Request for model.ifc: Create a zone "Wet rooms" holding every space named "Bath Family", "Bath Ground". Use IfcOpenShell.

First a look at what the model holds.

```python
import ifcopenshell

model = ifcopenshell.open("model.ifc")
print(model.schema)
seen = {}
for space in model.by_type("IfcSpace"):
    seen[space.LongName] = seen.get(space.LongName, 0) + 1
for name, count in sorted(seen.items(), key=str):
    print(count, "x", name)
print("zones:", [z.Name for z in model.by_type("IfcZone")][:20])
```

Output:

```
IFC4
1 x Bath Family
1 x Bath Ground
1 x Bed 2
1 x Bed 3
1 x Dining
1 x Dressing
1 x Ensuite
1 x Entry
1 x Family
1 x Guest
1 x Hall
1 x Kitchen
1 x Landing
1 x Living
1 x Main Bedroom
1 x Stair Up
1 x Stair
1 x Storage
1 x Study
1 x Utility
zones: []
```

```python
import ifcopenshell
import ifcopenshell.api.group
import ifcopenshell.api.root

model = ifcopenshell.open("model.ifc")

names = {"Bath Family", "Bath Ground"}
spaces = [s for s in model.by_type("IfcSpace") if s.LongName in names]

zone = ifcopenshell.api.root.create_entity(model, ifc_class="IfcZone", name="Wet rooms")
ifcopenshell.api.group.assign_group(model, products=spaces, group=zone)
print(len(spaces), "spaces in", zone.Name)

model.write("model_v2.ifc")
```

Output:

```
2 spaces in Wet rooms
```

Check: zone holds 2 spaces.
